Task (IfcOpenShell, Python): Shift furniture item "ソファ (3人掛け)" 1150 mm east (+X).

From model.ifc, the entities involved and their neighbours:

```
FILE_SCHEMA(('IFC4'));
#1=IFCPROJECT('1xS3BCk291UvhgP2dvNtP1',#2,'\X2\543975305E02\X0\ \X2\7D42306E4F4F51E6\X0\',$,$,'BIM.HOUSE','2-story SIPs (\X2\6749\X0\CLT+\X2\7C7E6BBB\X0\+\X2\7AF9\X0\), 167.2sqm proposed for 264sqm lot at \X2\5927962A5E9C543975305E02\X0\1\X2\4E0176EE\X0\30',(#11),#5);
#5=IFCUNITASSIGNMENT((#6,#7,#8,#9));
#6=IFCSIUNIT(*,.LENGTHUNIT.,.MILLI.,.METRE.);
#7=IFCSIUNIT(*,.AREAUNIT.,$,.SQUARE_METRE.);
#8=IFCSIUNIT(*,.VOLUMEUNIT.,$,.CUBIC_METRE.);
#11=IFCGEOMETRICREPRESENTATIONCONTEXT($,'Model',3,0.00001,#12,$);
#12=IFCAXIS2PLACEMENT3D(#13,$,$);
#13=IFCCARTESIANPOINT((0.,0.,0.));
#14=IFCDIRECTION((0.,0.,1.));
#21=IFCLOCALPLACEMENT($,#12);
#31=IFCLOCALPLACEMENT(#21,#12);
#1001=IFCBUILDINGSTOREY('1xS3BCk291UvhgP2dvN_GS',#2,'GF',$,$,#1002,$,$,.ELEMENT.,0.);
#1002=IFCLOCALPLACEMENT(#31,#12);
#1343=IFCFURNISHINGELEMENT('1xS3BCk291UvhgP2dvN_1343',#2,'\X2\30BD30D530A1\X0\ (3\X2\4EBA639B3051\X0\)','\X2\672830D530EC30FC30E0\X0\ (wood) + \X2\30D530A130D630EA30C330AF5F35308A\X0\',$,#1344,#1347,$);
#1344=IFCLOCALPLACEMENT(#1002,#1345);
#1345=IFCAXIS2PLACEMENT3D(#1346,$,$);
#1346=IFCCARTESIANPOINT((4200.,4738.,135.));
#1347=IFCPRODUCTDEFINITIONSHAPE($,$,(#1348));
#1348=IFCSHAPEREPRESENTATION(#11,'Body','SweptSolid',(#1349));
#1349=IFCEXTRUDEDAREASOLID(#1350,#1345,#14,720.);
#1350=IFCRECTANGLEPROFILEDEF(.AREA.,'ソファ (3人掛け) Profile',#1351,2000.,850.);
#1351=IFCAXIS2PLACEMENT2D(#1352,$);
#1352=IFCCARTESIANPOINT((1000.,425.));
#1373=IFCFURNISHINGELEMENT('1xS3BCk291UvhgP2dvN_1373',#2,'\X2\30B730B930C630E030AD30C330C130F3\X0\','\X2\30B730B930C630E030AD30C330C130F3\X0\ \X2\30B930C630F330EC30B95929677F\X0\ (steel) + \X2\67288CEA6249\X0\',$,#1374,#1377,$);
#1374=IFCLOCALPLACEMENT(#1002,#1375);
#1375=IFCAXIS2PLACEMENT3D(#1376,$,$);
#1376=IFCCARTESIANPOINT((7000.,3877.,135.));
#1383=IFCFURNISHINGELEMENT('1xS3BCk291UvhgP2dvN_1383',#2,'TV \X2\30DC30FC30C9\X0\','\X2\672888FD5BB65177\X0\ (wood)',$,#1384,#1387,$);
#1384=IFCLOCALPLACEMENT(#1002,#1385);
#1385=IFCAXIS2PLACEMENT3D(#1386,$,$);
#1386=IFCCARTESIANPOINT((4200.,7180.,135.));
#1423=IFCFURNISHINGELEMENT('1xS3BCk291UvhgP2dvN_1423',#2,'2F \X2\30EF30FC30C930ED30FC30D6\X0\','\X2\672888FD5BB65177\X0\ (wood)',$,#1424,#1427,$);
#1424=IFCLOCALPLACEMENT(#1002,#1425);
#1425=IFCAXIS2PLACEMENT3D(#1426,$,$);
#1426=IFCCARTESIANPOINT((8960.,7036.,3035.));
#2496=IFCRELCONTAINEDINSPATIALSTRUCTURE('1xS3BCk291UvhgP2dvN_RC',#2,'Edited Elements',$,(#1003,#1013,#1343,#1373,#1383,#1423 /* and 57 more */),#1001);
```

```python
import ifcopenshell
import ifcopenshell.api.geometry
import ifcopenshell.util.placement
import ifcopenshell.util.unit

model = ifcopenshell.open("model.ifc")
unit_scale = ifcopenshell.util.unit.calculate_unit_scale(model)

item = model.by_id(1343)
matrix = ifcopenshell.util.placement.get_local_placement(item.ObjectPlacement)
matrix[0, 3] += 1.15 / unit_scale
ifcopenshell.api.geometry.edit_object_placement(model, product=item, matrix=matrix, is_si=False)

print(ifcopenshell.util.placement.get_local_placement(item.ObjectPlacement).round(3) + 0.0)

model.write("model_updated.ifc")
```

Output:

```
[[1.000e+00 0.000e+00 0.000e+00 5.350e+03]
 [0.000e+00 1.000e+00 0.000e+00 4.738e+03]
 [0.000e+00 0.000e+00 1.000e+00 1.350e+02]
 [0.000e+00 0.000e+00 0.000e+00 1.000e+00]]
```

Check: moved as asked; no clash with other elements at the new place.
